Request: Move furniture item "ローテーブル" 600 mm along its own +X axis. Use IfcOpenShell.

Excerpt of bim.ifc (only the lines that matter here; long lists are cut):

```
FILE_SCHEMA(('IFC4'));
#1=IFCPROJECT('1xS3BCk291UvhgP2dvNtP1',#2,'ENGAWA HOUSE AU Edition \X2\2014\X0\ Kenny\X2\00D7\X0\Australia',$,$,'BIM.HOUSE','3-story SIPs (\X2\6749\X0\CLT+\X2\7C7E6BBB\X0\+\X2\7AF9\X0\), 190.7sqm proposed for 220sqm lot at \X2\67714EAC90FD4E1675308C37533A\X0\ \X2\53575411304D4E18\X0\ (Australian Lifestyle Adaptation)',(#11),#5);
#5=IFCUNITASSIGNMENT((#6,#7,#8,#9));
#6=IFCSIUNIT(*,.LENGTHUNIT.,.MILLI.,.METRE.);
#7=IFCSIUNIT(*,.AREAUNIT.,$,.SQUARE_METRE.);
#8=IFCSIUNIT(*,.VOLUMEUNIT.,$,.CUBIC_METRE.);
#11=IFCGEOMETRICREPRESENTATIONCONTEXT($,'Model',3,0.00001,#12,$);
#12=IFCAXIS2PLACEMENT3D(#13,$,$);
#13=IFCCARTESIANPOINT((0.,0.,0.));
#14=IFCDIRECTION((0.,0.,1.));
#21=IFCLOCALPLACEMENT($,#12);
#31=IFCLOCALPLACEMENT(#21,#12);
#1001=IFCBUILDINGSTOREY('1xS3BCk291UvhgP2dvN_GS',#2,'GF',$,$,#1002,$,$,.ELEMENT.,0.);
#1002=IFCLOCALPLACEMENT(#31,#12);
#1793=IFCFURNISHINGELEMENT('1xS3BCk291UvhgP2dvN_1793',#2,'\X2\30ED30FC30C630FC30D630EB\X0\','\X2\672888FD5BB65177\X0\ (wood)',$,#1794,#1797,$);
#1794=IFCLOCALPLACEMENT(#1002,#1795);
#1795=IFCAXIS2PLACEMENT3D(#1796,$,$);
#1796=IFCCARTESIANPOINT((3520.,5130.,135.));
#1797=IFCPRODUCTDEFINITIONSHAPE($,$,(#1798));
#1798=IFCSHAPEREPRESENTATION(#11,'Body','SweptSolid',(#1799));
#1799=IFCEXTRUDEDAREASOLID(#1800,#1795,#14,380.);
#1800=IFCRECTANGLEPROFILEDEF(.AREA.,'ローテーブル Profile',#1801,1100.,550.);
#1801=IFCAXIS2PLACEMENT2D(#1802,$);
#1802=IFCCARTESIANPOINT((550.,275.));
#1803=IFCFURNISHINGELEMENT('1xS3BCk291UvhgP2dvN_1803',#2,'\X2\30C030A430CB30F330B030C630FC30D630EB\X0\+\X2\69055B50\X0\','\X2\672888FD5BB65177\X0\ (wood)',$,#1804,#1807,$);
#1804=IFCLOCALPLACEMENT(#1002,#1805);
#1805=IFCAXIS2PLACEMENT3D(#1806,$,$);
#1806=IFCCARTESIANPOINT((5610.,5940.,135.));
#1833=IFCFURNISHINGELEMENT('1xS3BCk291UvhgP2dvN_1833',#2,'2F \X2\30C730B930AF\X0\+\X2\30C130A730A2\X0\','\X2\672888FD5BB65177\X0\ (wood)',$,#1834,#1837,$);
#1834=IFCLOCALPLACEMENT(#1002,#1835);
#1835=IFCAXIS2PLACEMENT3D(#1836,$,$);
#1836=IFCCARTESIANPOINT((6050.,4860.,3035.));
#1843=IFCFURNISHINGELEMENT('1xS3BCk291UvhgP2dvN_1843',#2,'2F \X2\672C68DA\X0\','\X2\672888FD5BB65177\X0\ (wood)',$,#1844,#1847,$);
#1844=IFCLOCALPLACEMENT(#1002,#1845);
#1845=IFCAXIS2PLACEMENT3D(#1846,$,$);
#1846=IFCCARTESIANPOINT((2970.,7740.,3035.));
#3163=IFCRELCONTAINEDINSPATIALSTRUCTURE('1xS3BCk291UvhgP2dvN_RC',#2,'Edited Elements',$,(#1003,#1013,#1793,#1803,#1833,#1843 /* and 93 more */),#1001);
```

```python
import ifcopenshell
import ifcopenshell.api.geometry
import ifcopenshell.util.placement
import ifcopenshell.util.unit

model = ifcopenshell.open("bim.ifc")
unit_scale = ifcopenshell.util.unit.calculate_unit_scale(model)

item = model.by_guid("1xS3BCk291UvhgP2dvN_1793")
matrix = ifcopenshell.util.placement.get_local_placement(item.ObjectPlacement)
matrix[:3, 3] += matrix[:3, 0] * 0.6 / unit_scale
ifcopenshell.api.geometry.edit_object_placement(model, product=item, matrix=matrix, is_si=False)

print(ifcopenshell.util.placement.get_local_placement(item.ObjectPlacement).round(3) + 0.0)

model.write("bim-out.ifc")
```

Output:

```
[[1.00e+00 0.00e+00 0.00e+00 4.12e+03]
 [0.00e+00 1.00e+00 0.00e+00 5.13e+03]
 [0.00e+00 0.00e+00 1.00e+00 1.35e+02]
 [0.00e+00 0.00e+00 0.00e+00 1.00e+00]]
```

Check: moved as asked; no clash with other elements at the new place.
